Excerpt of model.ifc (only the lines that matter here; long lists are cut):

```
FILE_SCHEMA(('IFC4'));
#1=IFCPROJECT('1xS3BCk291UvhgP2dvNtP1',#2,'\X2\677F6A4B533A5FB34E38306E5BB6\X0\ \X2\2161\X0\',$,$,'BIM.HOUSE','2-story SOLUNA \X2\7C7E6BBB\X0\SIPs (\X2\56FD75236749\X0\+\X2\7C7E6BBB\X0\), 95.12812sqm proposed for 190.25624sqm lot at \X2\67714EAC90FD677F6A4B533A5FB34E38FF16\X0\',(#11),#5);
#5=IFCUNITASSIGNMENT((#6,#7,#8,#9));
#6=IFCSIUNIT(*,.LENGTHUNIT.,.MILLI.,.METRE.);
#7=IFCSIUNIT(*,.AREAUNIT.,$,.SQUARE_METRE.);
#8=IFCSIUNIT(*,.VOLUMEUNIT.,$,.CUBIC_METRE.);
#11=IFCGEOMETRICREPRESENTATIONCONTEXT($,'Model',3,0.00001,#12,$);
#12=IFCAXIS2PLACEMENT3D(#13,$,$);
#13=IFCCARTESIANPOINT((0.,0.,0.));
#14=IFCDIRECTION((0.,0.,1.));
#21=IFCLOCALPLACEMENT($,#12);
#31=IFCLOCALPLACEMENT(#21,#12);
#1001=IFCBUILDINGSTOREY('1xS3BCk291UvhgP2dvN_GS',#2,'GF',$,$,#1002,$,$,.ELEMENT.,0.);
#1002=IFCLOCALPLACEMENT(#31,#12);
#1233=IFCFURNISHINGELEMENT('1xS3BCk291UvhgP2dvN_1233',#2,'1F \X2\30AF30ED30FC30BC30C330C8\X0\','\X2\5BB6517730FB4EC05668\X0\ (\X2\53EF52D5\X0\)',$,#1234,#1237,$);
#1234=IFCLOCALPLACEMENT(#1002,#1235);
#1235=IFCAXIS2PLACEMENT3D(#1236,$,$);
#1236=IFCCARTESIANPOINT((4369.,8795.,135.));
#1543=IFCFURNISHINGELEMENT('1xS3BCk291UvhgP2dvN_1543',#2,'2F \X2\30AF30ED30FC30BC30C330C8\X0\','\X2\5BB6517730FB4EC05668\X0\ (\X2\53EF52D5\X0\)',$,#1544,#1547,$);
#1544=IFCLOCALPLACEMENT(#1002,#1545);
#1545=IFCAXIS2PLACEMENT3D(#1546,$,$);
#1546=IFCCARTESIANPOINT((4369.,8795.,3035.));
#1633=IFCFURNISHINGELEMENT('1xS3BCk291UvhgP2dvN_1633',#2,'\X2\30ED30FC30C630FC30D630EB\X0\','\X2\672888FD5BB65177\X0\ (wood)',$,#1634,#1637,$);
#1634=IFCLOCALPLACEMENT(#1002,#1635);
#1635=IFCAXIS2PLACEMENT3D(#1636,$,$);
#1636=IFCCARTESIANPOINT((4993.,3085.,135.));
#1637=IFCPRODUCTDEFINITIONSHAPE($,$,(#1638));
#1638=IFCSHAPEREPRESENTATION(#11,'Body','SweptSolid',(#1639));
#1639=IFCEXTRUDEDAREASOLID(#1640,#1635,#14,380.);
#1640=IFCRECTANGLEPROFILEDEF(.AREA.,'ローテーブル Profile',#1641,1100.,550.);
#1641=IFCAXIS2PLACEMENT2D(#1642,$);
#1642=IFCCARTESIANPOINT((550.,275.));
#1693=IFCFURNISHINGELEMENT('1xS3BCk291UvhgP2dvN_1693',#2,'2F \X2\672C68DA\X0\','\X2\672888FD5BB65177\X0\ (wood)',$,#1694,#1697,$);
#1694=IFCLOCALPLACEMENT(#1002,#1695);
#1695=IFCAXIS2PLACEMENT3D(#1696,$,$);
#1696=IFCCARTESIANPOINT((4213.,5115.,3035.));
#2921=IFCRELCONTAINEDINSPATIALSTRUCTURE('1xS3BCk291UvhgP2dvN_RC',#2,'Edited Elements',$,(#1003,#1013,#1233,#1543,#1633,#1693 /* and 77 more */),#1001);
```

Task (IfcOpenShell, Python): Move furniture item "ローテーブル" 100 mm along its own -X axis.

```python
import ifcopenshell
import ifcopenshell.api.geometry
import ifcopenshell.util.placement
import ifcopenshell.util.unit

model = ifcopenshell.open("model.ifc")
unit_scale = ifcopenshell.util.unit.calculate_unit_scale(model)

item = model.by_id(1633)
matrix = ifcopenshell.util.placement.get_local_placement(item.ObjectPlacement)
matrix[:3, 3] -= matrix[:3, 0] * 0.1 / unit_scale
ifcopenshell.api.geometry.edit_object_placement(model, product=item, matrix=matrix, is_si=False)

print(ifcopenshell.util.placement.get_local_placement(item.ObjectPlacement).round(3) + 0.0)

model.write("model_updated.ifc")
```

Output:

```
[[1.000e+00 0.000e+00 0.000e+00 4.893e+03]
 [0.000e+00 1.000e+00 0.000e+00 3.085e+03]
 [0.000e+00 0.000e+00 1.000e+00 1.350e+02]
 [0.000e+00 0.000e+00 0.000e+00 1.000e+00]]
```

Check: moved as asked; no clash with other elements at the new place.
